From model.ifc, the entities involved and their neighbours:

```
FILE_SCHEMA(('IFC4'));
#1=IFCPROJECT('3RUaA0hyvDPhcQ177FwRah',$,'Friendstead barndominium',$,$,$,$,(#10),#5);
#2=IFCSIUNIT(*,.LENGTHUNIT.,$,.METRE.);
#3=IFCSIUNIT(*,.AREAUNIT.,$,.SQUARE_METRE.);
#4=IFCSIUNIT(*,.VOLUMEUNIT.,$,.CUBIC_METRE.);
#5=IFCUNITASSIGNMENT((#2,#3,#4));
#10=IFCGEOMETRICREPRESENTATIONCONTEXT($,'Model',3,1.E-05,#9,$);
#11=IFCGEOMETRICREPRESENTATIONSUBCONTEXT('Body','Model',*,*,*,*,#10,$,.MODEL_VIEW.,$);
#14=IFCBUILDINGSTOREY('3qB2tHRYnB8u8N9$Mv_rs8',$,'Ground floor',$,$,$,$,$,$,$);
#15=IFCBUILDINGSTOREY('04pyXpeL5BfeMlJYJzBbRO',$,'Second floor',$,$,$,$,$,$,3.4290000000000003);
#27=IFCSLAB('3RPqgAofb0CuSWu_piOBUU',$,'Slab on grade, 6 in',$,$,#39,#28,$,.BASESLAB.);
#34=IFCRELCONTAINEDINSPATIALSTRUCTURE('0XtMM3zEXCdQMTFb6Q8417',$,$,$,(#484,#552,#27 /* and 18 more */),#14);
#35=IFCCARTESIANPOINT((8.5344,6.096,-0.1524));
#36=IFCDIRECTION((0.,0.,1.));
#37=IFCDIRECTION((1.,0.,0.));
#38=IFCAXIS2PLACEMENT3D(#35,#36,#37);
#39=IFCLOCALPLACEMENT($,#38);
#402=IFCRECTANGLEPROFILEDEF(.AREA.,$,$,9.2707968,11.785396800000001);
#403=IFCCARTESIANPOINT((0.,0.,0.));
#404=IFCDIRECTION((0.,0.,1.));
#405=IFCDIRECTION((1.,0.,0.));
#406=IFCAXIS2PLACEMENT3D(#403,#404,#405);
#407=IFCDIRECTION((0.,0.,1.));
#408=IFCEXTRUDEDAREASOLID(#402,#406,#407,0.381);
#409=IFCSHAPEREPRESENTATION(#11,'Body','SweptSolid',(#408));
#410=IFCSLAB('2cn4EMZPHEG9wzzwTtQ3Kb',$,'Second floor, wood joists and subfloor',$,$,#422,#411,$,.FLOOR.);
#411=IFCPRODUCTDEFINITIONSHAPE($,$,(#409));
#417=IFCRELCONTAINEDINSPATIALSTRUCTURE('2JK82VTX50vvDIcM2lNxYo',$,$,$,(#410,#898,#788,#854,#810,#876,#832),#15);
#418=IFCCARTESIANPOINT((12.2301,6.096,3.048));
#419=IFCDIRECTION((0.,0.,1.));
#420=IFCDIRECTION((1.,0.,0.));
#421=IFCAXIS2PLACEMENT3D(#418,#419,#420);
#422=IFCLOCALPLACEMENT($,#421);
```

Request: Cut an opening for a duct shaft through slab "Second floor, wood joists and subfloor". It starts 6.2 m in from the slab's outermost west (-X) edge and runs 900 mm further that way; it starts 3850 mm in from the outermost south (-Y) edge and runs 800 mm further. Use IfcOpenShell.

```python
import numpy as np
import ifcopenshell
import ifcopenshell.api.feature
import ifcopenshell.api.geometry
import ifcopenshell.api.root
import ifcopenshell.geom
import ifcopenshell.util.placement
import ifcopenshell.util.representation
import ifcopenshell.util.shape
import ifcopenshell.util.unit

model = ifcopenshell.open("model.ifc")
unit_scale = ifcopenshell.util.unit.calculate_unit_scale(model)
settings = ifcopenshell.geom.settings()


def volume(element):
    """Net volume in cubic metres, openings subtracted."""
    shape = ifcopenshell.geom.create_shape(settings, element)
    return ifcopenshell.util.shape.get_volume(shape.geometry)


slab = model.by_id(410)
before = volume(slab)

# Extent in the slab's own axes, in metres. The edges named are its -X and -Y sides.
slab_shape = ifcopenshell.geom.create_shape(settings, slab)
vertices = ifcopenshell.util.shape.get_vertices(slab_shape.geometry)
x_min, y_min, bottom = vertices.min(axis=0)
top = vertices[:, 2].max()

opening = ifcopenshell.api.root.create_entity(model, ifc_class="IfcOpeningElement", name="Duct shaft opening", predefined_type="OPENING")
context = ifcopenshell.util.representation.get_context(model, "Model", "Body", "MODEL_VIEW")
width, depth = 0.9, 0.8
outline = [(0.0, 0.0), (width, 0.0), (width, depth), (0.0, depth), (0.0, 0.0)]
# Overshoot both faces by 50 mm so the cut is clean.
shape = ifcopenshell.api.geometry.add_slab_representation(
    model, context=context, depth=top - bottom + 0.1, polyline=outline
)
ifcopenshell.api.geometry.assign_representation(model, product=opening, representation=shape)

matrix = ifcopenshell.util.placement.get_local_placement(slab.ObjectPlacement)
matrix[:, 3] = matrix @ np.append(np.array([x_min + 6.2, y_min + 3.85, bottom - 0.05]) / unit_scale, 1.0)
ifcopenshell.api.geometry.edit_object_placement(model, product=opening, matrix=matrix, is_si=False)
ifcopenshell.api.feature.add_feature(model, feature=opening, element=slab)

after = volume(slab)

print(f"slab volume {before:.3f} -> {after:.3f} m3")

model.write("model_updated.ifc")
```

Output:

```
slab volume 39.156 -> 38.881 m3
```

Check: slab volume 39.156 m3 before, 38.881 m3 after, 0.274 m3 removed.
